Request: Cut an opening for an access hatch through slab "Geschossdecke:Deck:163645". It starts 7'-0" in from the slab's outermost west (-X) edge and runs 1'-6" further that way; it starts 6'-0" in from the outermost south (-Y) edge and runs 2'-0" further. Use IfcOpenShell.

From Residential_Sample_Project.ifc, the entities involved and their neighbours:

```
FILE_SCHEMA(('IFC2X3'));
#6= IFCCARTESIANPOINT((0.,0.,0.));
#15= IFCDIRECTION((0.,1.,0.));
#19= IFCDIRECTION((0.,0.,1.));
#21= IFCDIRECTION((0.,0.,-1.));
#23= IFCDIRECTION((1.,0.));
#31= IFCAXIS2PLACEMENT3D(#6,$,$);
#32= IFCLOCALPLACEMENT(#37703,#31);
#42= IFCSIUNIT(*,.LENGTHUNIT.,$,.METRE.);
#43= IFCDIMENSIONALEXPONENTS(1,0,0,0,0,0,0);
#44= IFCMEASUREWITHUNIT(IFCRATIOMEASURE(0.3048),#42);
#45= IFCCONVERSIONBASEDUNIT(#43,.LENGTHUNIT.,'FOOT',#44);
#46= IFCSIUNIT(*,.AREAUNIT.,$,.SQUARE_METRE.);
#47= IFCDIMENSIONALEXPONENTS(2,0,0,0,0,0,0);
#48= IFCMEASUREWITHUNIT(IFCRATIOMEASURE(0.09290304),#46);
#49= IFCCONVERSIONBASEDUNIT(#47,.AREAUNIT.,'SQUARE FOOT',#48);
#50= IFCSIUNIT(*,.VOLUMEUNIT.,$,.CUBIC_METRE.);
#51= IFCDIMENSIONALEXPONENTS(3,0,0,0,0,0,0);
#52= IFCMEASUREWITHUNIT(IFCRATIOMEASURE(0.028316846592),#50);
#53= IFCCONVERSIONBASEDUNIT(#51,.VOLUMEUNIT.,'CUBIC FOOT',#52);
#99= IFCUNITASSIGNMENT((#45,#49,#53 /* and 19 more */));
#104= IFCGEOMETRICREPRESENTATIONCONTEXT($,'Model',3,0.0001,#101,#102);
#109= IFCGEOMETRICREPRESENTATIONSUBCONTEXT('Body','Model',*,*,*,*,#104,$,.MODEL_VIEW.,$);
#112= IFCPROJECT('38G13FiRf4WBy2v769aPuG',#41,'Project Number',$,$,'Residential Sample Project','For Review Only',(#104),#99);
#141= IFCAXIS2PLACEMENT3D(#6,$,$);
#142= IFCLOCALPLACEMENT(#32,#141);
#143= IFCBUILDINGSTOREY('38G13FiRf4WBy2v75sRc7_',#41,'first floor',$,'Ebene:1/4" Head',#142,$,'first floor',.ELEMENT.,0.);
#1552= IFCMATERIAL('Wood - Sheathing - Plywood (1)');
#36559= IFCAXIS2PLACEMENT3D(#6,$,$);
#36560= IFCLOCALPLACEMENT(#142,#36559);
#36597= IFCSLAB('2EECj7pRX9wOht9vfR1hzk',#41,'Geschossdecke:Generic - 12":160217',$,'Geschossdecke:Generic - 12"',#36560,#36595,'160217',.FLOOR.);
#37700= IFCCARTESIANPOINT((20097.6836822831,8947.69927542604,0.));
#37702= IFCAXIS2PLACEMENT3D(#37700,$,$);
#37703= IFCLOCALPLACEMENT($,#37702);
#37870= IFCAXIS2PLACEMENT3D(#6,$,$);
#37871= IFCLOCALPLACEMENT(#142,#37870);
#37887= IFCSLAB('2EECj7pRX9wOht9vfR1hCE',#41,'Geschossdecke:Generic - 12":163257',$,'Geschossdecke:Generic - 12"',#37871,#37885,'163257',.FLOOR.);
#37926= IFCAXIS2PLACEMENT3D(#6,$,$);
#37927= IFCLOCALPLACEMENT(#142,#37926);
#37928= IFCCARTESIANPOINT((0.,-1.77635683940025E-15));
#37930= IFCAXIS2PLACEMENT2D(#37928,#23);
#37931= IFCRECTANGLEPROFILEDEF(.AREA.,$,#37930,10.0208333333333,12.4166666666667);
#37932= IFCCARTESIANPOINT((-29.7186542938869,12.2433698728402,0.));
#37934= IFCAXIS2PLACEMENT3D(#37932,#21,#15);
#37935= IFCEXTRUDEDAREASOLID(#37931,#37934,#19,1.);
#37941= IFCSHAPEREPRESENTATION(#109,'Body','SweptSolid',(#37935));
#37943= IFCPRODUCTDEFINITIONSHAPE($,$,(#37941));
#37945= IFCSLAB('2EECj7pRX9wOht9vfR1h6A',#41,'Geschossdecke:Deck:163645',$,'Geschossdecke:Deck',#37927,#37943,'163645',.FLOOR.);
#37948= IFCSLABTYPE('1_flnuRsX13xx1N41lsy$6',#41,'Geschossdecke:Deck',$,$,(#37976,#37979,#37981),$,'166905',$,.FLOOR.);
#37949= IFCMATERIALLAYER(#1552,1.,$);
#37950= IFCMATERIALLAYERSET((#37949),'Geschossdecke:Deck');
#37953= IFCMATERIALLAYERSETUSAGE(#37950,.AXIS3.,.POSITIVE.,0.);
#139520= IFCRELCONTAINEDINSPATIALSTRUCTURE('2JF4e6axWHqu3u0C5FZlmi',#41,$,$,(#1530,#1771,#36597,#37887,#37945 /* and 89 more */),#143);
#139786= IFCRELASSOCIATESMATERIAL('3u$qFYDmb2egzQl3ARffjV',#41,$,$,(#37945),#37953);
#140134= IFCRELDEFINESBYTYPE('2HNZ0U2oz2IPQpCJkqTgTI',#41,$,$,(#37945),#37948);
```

```python
import numpy as np
import ifcopenshell
import ifcopenshell.api.feature
import ifcopenshell.api.geometry
import ifcopenshell.api.root
import ifcopenshell.geom
import ifcopenshell.util.placement
import ifcopenshell.util.representation
import ifcopenshell.util.shape
import ifcopenshell.util.unit

model = ifcopenshell.open("Residential_Sample_Project.ifc")
unit_scale = ifcopenshell.util.unit.calculate_unit_scale(model)
settings = ifcopenshell.geom.settings()


def volume(element):
    """Net volume in cubic metres, openings subtracted."""
    shape = ifcopenshell.geom.create_shape(settings, element)
    return ifcopenshell.util.shape.get_volume(shape.geometry)


slab = model.by_guid("2EECj7pRX9wOht9vfR1h6A")
before = volume(slab)

# Extent in the slab's own axes, in metres. The edges named are its -X and -Y sides.
slab_shape = ifcopenshell.geom.create_shape(settings, slab)
vertices = ifcopenshell.util.shape.get_vertices(slab_shape.geometry)
x_min, y_min, bottom = vertices.min(axis=0)
top = vertices[:, 2].max()

opening = ifcopenshell.api.root.create_entity(model, ifc_class="IfcOpeningElement", name="Access hatch opening")
context = ifcopenshell.util.representation.get_context(model, "Model", "Body", "MODEL_VIEW")
width, depth = 0.4572, 0.6096
outline = [(0.0, 0.0), (width, 0.0), (width, depth), (0.0, depth), (0.0, 0.0)]
# Overshoot both faces by 50 mm so the cut is clean.
shape = ifcopenshell.api.geometry.add_slab_representation(
    model, context=context, depth=top - bottom + 0.1, polyline=outline
)
ifcopenshell.api.geometry.assign_representation(model, product=opening, representation=shape)

matrix = ifcopenshell.util.placement.get_local_placement(slab.ObjectPlacement)
matrix[:, 3] = matrix @ np.append(np.array([x_min + 2.1336, y_min + 1.8288, bottom - 0.05]) / unit_scale, 1.0)
ifcopenshell.api.geometry.edit_object_placement(model, product=opening, matrix=matrix, is_si=False)
ifcopenshell.api.feature.add_feature(model, feature=opening, element=slab)

after = volume(slab)

print(f"slab volume {before:.3f} -> {after:.3f} m3")

model.write("Residential_Sample_Project_updated.ifc")
```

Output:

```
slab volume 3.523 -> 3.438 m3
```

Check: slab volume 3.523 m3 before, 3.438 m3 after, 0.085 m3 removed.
